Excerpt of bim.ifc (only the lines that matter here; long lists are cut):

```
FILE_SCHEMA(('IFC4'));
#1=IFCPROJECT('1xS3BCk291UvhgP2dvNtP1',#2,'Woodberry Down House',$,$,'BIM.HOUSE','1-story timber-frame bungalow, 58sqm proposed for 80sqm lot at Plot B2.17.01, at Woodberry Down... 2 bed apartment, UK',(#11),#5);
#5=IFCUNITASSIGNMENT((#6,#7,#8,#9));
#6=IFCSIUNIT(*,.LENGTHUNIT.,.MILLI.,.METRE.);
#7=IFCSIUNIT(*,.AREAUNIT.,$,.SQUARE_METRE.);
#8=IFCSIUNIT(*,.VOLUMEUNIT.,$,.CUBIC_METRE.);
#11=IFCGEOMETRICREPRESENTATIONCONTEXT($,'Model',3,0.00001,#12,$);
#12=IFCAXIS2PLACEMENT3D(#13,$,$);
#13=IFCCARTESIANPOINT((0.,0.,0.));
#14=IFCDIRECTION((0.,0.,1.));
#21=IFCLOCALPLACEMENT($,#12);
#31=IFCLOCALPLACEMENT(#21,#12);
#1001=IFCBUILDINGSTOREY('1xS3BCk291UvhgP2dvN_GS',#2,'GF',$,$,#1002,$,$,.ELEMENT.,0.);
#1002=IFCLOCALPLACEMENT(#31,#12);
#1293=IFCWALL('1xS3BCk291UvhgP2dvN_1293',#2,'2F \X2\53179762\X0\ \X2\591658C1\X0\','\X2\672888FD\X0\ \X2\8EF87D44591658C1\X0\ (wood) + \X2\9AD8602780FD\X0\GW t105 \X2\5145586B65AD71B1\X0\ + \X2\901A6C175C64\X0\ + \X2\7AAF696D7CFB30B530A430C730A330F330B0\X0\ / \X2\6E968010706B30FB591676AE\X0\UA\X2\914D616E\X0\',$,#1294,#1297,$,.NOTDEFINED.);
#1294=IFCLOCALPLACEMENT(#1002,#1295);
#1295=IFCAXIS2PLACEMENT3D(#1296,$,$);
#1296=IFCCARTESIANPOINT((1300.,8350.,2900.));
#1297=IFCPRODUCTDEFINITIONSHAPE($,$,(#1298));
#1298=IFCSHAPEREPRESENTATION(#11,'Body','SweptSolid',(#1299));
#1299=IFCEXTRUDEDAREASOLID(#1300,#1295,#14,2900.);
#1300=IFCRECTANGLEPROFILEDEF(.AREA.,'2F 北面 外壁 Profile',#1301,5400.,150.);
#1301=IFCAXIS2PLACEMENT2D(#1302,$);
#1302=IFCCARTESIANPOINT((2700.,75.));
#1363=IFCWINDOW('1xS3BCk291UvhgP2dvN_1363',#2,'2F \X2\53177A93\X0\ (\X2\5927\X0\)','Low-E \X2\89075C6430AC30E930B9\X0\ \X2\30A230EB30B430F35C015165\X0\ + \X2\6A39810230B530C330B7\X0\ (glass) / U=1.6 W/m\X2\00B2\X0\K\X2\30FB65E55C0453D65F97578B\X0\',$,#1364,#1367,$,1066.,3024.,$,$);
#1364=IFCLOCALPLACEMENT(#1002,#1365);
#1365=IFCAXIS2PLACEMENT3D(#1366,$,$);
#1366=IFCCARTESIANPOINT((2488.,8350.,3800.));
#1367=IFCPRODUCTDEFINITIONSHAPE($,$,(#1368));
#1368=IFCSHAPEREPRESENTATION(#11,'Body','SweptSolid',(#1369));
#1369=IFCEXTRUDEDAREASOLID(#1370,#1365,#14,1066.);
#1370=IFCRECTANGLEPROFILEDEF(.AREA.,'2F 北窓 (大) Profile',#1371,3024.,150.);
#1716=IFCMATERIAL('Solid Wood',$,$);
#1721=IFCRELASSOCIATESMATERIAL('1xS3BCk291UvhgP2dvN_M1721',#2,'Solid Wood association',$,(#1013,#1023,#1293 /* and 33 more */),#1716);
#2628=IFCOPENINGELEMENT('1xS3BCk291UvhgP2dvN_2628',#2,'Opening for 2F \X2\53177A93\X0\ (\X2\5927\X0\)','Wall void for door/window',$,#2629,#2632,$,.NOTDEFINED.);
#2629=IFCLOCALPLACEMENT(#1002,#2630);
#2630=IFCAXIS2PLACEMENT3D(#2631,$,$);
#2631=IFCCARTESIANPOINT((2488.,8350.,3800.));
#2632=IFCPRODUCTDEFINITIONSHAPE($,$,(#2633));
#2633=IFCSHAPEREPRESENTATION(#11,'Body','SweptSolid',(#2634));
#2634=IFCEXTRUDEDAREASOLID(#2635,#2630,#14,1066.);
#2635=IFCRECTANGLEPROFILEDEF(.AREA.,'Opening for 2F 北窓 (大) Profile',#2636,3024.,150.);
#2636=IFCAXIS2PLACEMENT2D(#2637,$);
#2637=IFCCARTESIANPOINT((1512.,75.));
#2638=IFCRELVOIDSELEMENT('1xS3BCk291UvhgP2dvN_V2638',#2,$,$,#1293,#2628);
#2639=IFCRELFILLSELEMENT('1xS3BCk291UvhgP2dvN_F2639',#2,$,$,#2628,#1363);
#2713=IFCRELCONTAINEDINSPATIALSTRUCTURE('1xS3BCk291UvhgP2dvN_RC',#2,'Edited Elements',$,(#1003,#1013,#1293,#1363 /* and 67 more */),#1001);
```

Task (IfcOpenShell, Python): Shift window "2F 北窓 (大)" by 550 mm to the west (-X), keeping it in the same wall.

```python
import ifcopenshell
import ifcopenshell.api.geometry
import ifcopenshell.util.placement

model = ifcopenshell.open("bim.ifc")

window = model.by_id(1363)
opening = window.FillsVoids[0].RelatingOpeningElement
wall = opening.VoidsElements[0].RelatingBuildingElement

wall_matrix = ifcopenshell.util.placement.get_local_placement(wall.ObjectPlacement)
shift = wall_matrix[:3, 0] * -550.0
before = ifcopenshell.util.placement.get_local_placement(window.ObjectPlacement)[:3, 3].copy()

# The window is not placed relative to its opening, so move both.
for product in (opening, window):
    matrix = ifcopenshell.util.placement.get_local_placement(product.ObjectPlacement)
    matrix[:3, 3] += shift
    ifcopenshell.api.geometry.edit_object_placement(model, product=product, matrix=matrix, is_si=False)

after = ifcopenshell.util.placement.get_local_placement(window.ObjectPlacement)[:3, 3]
print("window moved by", (after - before).round(3) + 0.0)

model.write("bim_updated.ifc")
```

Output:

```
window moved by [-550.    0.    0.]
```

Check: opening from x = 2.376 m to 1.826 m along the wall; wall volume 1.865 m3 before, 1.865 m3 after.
